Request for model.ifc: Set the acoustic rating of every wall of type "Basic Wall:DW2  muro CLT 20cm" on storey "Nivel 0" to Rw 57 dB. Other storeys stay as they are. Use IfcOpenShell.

First a look at what the model holds.

```python
import ifcopenshell
import ifcopenshell.util.element

model = ifcopenshell.open("model.ifc")
print(model.schema)
storey = next(s for s in model.by_type("IfcBuildingStorey") if s.Name == "Nivel 0")
walls = [e for e in ifcopenshell.util.element.get_decomposition(storey) if e.is_a("IfcWall")]
seen = {}
for e in walls:
    element_type = ifcopenshell.util.element.get_type(e)
    key = (element_type.Name if element_type != e and element_type else None, ifcopenshell.util.element.get_pset(e, "Pset_WallCommon", "AcousticRating"))
    seen[key] = seen.get(key, 0) + 1
for (name, value), count in sorted(seen.items(), key=str):
    print(count, "x", name, "|", value)
```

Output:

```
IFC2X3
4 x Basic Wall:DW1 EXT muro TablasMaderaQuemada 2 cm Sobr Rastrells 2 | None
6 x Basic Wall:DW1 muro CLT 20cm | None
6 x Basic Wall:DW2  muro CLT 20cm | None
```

```python
import ifcopenshell
import ifcopenshell.api.pset
import ifcopenshell.util.element

model = ifcopenshell.open("model.ifc")

storey = next(s for s in model.by_type("IfcBuildingStorey") if s.Name == "Nivel 0")
walls = [e for e in ifcopenshell.util.element.get_decomposition(storey) if e.is_a("IfcWall")]

count = 0
for e in walls:
    element_type = ifcopenshell.util.element.get_type(e)
    if element_type in (None, e) or element_type.Name != "Basic Wall:DW2  muro CLT 20cm":
        continue
    # add_pset returns the element's existing set when there is one.
    pset = ifcopenshell.api.pset.add_pset(model, product=e, name="Pset_WallCommon")
    ifcopenshell.api.pset.edit_pset(model, pset=pset, properties={"AcousticRating": "Rw 57 dB"})
    count += 1

print(count, "walls updated")

model.write("model_v2.ifc")
```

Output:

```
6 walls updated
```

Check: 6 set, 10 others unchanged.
